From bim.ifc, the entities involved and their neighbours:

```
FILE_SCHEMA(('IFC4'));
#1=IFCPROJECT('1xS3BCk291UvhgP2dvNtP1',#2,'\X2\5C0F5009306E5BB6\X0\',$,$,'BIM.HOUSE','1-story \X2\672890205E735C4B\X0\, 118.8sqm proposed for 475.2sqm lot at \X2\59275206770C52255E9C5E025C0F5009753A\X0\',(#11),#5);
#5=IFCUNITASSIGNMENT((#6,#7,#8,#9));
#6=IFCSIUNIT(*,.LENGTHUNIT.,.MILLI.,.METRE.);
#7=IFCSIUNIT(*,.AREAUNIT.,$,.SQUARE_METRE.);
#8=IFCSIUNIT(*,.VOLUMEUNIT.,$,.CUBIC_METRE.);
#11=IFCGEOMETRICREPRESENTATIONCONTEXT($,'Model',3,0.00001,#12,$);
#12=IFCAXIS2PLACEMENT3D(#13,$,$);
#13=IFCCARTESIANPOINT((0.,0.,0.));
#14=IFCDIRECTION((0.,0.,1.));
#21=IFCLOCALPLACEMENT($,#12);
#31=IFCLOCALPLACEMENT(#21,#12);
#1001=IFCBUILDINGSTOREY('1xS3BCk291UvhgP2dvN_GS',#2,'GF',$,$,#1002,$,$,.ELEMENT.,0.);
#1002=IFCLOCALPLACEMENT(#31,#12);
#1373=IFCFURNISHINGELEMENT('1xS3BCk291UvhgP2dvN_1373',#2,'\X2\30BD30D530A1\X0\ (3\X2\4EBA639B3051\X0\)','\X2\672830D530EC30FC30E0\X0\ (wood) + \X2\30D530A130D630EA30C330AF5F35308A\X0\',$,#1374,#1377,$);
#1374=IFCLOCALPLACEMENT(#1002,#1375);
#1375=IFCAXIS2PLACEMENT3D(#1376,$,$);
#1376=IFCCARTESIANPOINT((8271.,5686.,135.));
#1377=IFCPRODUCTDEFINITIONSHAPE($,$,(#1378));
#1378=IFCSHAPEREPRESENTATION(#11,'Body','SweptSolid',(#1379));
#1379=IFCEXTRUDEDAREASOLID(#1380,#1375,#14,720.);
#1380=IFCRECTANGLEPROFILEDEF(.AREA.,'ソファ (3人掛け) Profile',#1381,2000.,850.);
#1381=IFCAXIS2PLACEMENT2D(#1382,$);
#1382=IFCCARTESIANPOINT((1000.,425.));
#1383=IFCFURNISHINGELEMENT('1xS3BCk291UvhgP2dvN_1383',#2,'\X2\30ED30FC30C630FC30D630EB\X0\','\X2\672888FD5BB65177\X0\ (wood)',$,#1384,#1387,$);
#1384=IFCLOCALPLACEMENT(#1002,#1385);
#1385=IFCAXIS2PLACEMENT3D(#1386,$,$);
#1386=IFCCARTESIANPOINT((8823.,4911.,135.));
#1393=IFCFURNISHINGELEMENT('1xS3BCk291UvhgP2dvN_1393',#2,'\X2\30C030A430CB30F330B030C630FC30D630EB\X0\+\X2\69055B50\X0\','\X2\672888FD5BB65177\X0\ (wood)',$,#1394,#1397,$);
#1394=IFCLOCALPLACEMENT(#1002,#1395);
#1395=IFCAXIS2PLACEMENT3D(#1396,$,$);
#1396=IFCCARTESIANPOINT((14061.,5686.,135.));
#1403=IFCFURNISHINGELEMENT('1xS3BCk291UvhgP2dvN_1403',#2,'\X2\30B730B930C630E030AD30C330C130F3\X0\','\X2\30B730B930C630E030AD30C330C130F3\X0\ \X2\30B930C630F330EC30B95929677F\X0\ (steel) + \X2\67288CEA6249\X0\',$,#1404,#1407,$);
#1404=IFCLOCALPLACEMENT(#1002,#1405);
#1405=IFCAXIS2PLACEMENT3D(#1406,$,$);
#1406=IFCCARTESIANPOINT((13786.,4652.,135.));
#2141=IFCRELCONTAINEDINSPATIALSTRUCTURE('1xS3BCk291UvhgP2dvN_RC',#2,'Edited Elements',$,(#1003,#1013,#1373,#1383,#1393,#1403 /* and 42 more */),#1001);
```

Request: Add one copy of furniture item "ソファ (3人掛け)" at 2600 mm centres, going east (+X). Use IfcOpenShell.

```python
import numpy as np
import ifcopenshell
import ifcopenshell.api.geometry
import ifcopenshell.api.root
import ifcopenshell.util.element
import ifcopenshell.util.placement

model = ifcopenshell.open("bim.ifc")


def reuse_history(source, copy):
    """copy_class also copies each property set's owner history, people and application; keep the originals."""
    for rel in copy.IsDefinedBy:
        if rel.is_a("IfcRelDefinesByProperties") and (history := rel.RelatingPropertyDefinition.OwnerHistory):
            rel.RelatingPropertyDefinition.OwnerHistory = source.OwnerHistory
            ifcopenshell.util.element.remove_deep2(model, history)


source = model.by_id(1373)
base = ifcopenshell.util.placement.get_local_placement(source.ObjectPlacement)
step = np.array([1.0, 0.0, 0.0]) * 2600.0

for i in range(1, 2):
    copy = ifcopenshell.api.root.copy_class(model, product=source)
    copy.Representation = ifcopenshell.util.element.copy_deep(
        model, source.Representation, exclude=["IfcGeometricRepresentationContext", "IfcRepresentationMap"]
    )
    reuse_history(source, copy)
    matrix = base.copy()
    matrix[:3, 3] += i * step
    print("added at", matrix[:3, 3].round(3) + 0.0)
    ifcopenshell.api.geometry.edit_object_placement(model, product=copy, matrix=matrix, is_si=False)

model.write("bim_edited.ifc")
```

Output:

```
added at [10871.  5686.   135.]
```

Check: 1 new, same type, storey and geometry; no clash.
